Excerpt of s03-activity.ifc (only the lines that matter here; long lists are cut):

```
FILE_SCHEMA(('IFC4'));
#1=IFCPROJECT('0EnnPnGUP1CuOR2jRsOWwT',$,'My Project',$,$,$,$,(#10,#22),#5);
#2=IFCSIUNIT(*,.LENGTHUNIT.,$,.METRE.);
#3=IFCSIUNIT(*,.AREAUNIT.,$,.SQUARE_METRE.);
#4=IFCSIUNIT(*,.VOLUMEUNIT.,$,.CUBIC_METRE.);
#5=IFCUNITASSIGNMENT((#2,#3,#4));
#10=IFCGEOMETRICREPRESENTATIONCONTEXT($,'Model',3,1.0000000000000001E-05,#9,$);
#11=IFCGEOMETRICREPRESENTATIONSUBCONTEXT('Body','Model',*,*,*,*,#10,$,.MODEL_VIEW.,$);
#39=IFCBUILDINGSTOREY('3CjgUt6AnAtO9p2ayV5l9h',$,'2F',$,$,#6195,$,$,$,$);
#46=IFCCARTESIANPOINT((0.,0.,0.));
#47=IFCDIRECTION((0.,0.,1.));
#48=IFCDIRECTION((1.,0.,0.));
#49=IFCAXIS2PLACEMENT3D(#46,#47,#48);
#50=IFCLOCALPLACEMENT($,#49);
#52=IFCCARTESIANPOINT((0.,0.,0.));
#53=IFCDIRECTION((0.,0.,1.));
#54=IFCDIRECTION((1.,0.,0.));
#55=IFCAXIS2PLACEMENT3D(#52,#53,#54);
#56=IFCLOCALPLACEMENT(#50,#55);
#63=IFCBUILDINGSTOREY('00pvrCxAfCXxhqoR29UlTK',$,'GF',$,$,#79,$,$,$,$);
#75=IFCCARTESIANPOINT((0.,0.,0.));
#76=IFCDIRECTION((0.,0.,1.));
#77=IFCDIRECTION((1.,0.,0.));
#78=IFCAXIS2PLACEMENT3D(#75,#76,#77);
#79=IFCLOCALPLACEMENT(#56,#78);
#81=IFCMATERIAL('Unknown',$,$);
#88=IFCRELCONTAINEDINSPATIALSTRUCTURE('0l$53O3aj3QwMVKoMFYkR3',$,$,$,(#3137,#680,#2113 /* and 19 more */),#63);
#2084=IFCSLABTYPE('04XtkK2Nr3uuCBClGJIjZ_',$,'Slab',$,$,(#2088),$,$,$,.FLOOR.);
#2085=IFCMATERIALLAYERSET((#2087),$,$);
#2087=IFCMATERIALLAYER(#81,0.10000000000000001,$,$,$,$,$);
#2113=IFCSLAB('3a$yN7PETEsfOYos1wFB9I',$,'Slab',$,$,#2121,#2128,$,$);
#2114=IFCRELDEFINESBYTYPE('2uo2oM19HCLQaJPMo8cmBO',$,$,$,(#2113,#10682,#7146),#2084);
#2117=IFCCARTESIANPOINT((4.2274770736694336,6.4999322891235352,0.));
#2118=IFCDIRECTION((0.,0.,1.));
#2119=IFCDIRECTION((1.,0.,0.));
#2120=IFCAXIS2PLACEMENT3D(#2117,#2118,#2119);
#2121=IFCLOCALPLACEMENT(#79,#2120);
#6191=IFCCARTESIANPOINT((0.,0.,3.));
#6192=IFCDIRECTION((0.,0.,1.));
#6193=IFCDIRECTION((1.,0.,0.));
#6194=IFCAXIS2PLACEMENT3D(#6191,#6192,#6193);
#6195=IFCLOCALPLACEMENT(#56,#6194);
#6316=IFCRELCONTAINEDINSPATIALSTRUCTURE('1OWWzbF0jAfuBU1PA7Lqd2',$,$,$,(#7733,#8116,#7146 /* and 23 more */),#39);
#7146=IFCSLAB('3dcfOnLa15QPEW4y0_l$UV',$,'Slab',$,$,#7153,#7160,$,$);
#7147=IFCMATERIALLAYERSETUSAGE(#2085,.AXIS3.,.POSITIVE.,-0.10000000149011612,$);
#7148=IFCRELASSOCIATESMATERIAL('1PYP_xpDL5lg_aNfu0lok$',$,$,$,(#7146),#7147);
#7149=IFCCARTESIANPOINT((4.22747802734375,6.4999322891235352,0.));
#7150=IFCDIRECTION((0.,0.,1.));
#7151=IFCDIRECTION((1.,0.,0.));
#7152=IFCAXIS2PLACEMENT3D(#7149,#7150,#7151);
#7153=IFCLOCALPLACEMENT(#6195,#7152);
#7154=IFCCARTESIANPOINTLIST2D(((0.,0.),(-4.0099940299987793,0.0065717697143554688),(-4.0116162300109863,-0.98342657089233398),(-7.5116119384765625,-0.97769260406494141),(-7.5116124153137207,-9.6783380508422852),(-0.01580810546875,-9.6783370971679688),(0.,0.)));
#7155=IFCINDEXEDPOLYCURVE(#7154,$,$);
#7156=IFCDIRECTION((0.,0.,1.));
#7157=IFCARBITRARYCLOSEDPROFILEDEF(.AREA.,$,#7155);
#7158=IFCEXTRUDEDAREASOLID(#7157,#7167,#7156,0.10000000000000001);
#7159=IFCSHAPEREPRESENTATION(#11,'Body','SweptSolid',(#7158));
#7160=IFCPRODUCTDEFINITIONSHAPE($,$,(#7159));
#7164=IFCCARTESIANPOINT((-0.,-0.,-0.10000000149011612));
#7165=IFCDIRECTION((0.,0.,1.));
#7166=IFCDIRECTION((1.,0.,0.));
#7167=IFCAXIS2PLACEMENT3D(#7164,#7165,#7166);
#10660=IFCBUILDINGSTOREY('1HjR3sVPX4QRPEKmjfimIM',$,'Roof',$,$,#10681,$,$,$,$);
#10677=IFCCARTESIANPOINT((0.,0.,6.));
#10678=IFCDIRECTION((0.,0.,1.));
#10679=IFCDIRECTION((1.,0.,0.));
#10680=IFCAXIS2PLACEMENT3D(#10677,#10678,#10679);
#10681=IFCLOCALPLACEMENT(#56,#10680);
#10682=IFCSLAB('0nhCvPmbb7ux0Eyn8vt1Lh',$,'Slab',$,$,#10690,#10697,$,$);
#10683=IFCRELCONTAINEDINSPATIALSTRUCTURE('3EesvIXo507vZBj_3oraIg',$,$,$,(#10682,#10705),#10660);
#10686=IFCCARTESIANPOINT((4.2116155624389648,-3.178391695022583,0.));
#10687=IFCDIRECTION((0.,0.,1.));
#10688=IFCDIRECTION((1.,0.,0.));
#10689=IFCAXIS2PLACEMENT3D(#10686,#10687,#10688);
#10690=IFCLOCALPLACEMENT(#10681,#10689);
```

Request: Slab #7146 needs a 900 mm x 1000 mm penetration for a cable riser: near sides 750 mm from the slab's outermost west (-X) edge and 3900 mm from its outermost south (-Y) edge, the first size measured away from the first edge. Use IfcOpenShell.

```python
import numpy as np
import ifcopenshell
import ifcopenshell.api.feature
import ifcopenshell.api.geometry
import ifcopenshell.api.root
import ifcopenshell.geom
import ifcopenshell.util.placement
import ifcopenshell.util.representation
import ifcopenshell.util.shape
import ifcopenshell.util.unit

model = ifcopenshell.open("s03-activity.ifc")
unit_scale = ifcopenshell.util.unit.calculate_unit_scale(model)
settings = ifcopenshell.geom.settings()


def volume(element):
    """Net volume in cubic metres, openings subtracted."""
    shape = ifcopenshell.geom.create_shape(settings, element)
    return ifcopenshell.util.shape.get_volume(shape.geometry)


slab = model.by_guid("3dcfOnLa15QPEW4y0_l$UV")
before = volume(slab)

# Extent in the slab's own axes, in metres. The edges named are its -X and -Y sides.
slab_shape = ifcopenshell.geom.create_shape(settings, slab)
vertices = ifcopenshell.util.shape.get_vertices(slab_shape.geometry)
x_min, y_min, bottom = vertices.min(axis=0)
top = vertices[:, 2].max()

opening = ifcopenshell.api.root.create_entity(model, ifc_class="IfcOpeningElement", name="Cable riser opening", predefined_type="OPENING")
context = ifcopenshell.util.representation.get_context(model, "Model", "Body", "MODEL_VIEW")
width, depth = 0.9, 1
outline = [(0.0, 0.0), (width, 0.0), (width, depth), (0.0, depth), (0.0, 0.0)]
# Overshoot both faces by 50 mm so the cut is clean.
shape = ifcopenshell.api.geometry.add_slab_representation(
    model, context=context, depth=top - bottom + 0.1, polyline=outline
)
ifcopenshell.api.geometry.assign_representation(model, product=opening, representation=shape)

matrix = ifcopenshell.util.placement.get_local_placement(slab.ObjectPlacement)
matrix[:, 3] = matrix @ np.append(np.array([x_min + 0.75, y_min + 3.9, bottom - 0.05]) / unit_scale, 1.0)
ifcopenshell.api.geometry.edit_object_placement(model, product=opening, matrix=matrix, is_si=False)
ifcopenshell.api.feature.add_feature(model, feature=opening, element=slab)

after = volume(slab)

print(f"slab volume {before:.3f} -> {after:.3f} m3")

model.write("s03-activity_v2.ifc")
```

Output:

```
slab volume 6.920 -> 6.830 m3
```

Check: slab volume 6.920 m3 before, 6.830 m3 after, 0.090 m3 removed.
